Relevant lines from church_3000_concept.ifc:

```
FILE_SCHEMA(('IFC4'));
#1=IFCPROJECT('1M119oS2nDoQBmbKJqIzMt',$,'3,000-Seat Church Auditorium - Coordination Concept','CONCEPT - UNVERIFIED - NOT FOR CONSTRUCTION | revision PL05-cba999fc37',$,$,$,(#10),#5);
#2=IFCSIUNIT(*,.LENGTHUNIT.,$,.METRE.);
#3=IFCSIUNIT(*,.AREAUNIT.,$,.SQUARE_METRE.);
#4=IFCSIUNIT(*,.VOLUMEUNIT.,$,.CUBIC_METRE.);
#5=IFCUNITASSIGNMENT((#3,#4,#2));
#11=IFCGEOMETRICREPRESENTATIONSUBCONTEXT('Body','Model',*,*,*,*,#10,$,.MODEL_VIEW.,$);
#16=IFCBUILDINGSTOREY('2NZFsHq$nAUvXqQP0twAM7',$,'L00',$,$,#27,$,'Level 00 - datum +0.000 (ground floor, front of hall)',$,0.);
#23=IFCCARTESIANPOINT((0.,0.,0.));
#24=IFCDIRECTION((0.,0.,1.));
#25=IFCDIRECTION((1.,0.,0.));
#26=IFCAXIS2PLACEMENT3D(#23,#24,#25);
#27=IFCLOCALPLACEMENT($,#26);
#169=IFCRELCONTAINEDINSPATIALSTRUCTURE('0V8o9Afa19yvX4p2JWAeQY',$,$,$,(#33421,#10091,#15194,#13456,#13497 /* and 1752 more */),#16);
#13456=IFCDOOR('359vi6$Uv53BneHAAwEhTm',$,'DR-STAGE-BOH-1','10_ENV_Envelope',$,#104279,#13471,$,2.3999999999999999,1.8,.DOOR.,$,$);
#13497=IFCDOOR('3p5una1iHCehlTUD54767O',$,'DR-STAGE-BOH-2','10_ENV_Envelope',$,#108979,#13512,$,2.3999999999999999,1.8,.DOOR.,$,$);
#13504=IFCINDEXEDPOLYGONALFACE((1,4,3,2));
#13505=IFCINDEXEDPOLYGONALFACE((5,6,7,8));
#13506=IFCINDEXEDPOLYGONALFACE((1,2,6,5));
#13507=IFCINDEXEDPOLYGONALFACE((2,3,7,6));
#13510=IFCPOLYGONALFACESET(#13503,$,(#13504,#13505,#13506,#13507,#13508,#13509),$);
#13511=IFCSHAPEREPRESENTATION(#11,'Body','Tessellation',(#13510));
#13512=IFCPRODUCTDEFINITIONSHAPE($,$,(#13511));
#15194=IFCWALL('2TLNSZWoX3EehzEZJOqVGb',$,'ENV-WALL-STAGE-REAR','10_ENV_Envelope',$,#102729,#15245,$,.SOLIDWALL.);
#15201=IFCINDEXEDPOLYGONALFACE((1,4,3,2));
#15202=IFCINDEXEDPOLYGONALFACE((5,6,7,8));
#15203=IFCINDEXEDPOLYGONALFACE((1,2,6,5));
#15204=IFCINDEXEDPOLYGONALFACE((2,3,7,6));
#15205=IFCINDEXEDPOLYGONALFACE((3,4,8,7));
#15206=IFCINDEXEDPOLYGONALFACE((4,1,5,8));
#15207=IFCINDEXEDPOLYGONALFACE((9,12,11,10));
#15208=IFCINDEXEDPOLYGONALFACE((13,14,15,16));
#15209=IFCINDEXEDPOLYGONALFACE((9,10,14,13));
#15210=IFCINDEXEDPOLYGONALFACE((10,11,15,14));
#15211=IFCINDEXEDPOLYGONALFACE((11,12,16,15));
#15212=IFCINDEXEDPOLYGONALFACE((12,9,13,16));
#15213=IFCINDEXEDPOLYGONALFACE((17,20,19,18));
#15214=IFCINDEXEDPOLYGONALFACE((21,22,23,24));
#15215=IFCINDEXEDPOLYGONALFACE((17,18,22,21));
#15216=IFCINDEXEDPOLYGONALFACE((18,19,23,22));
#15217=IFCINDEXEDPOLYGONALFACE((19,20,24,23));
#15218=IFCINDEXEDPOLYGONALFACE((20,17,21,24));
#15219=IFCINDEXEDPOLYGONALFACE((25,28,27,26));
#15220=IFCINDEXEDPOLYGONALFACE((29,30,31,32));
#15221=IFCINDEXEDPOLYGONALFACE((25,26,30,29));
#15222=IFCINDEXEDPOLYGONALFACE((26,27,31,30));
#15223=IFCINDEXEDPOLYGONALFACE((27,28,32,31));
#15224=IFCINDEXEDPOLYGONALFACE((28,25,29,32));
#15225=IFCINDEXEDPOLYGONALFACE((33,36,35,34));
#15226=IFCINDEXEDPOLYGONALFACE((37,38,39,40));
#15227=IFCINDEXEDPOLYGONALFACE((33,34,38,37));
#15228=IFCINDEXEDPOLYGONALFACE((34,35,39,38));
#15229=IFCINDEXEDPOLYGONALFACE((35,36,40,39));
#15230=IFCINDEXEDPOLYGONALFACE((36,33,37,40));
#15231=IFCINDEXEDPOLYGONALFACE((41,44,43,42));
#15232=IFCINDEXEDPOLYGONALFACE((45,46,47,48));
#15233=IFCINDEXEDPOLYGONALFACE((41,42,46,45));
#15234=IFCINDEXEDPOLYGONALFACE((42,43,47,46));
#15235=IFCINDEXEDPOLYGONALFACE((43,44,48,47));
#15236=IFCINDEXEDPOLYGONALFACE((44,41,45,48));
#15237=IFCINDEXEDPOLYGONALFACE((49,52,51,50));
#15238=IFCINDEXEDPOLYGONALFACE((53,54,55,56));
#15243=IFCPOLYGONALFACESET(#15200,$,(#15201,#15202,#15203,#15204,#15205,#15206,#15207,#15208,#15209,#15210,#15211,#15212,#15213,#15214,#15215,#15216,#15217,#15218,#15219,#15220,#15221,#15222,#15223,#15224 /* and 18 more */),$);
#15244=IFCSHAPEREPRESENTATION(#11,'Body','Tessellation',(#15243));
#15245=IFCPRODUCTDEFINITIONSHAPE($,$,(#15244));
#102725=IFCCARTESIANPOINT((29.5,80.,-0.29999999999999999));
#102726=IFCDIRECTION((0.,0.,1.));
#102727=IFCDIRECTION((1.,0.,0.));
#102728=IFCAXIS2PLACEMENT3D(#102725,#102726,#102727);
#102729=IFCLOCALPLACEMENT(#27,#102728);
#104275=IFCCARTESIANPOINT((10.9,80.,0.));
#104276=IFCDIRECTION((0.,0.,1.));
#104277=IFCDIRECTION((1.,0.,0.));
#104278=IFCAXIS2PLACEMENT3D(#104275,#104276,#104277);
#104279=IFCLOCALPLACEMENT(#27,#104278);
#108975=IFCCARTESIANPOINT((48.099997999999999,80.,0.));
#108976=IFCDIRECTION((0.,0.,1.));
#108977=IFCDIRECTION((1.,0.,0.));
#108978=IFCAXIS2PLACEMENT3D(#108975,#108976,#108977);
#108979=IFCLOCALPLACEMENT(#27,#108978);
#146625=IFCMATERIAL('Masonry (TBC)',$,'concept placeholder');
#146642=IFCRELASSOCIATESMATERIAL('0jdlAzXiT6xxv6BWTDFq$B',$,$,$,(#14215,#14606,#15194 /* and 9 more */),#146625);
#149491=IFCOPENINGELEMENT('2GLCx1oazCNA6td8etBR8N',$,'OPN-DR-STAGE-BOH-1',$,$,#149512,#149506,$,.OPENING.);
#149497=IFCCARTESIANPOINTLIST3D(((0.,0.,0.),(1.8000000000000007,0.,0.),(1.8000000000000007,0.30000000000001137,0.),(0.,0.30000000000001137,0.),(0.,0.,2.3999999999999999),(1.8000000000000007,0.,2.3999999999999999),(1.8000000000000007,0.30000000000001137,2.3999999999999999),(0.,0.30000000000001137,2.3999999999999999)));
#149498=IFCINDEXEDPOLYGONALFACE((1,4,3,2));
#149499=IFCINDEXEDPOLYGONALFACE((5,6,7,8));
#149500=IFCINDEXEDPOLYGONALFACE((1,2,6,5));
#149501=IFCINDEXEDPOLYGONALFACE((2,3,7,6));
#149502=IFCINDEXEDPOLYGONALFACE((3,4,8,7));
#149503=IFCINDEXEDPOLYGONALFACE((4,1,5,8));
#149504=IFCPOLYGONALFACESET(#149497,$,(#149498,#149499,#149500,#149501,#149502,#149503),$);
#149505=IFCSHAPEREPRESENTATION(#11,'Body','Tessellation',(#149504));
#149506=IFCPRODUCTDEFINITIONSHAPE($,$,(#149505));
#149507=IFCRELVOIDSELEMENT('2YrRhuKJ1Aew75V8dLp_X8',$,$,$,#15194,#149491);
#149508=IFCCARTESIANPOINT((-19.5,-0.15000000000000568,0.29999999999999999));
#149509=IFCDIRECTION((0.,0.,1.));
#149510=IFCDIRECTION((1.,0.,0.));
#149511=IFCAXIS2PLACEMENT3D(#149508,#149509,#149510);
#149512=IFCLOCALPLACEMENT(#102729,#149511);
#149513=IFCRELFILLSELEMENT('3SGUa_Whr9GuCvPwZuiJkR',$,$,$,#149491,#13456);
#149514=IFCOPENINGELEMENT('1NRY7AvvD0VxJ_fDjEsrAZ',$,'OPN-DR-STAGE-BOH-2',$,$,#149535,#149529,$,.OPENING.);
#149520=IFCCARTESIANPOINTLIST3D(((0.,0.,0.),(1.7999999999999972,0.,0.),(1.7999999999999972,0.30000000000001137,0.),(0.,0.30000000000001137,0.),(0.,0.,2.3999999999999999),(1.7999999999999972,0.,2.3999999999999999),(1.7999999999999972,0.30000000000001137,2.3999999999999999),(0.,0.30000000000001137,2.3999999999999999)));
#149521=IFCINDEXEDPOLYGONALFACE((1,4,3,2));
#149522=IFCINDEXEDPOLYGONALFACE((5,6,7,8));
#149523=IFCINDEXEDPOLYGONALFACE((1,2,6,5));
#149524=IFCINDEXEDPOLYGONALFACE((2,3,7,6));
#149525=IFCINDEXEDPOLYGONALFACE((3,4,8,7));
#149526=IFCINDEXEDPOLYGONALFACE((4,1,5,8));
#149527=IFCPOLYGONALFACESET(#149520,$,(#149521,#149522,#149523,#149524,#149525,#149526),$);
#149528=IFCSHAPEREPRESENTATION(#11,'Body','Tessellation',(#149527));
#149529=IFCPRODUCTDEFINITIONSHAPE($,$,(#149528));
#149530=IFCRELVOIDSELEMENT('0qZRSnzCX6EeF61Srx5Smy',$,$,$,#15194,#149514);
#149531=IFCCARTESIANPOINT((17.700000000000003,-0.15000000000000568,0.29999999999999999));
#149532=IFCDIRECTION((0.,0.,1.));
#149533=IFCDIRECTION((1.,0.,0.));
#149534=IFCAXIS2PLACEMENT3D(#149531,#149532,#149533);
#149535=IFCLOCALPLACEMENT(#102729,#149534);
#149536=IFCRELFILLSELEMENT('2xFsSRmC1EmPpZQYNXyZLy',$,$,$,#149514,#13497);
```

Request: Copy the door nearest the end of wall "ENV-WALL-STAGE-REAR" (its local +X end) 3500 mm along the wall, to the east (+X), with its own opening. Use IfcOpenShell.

```python
import ifcopenshell
import ifcopenshell.api.feature
import ifcopenshell.api.geometry
import ifcopenshell.api.root
import ifcopenshell.geom
import ifcopenshell.util.element
import ifcopenshell.util.placement
import ifcopenshell.util.shape
import ifcopenshell.util.unit

model = ifcopenshell.open("church_3000_concept.ifc")
unit_scale = ifcopenshell.util.unit.calculate_unit_scale(model)
settings = ifcopenshell.geom.settings()


def volume(element):
    """Net volume in cubic metres, openings subtracted."""
    shape = ifcopenshell.geom.create_shape(settings, element)
    return ifcopenshell.util.shape.get_volume(shape.geometry)


door = model.by_id(13497)
opening = door.FillsVoids[0].RelatingOpeningElement
wall = opening.VoidsElements[0].RelatingBuildingElement
before = volume(wall)
shift = ifcopenshell.util.placement.get_local_placement(wall.ObjectPlacement)[:3, 0] * 3.5 / unit_scale

# copy_class copies the void relationship, type, container and properties, but no geometry.
new_opening = ifcopenshell.api.root.copy_class(model, product=opening)
new_opening.Representation = ifcopenshell.util.element.copy_deep(
    model, opening.Representation, exclude=["IfcGeometricRepresentationContext", "IfcRepresentationMap"]
)
new_door = ifcopenshell.api.root.copy_class(model, product=door)
new_door.Representation = ifcopenshell.util.element.copy_deep(
    model, door.Representation, exclude=["IfcGeometricRepresentationContext", "IfcRepresentationMap"]
)
ifcopenshell.api.feature.add_filling(model, opening=new_opening, element=new_door)

for old, new in ((opening, new_opening), (door, new_door)):
    matrix = ifcopenshell.util.placement.get_local_placement(old.ObjectPlacement)
    matrix[:3, 3] += shift
    ifcopenshell.api.geometry.edit_object_placement(model, product=new, matrix=matrix, is_si=False)

after = volume(wall)

print(f"wall volume {before:.3f} -> {after:.3f} m3")

model.write("church_3000_concept_rev.ifc")
```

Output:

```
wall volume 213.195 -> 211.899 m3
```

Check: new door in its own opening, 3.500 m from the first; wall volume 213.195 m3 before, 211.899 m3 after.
